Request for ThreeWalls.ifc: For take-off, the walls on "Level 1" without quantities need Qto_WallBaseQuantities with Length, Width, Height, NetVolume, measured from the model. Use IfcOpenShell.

First a look at what the model holds.

```python
import ifcopenshell
import ifcopenshell.util.element
import ifcopenshell.util.unit

model = ifcopenshell.open("ThreeWalls.ifc")
print(model.schema)
for unit_type in ("LENGTHUNIT", "AREAUNIT", "VOLUMEUNIT"):
    print(unit_type, ifcopenshell.util.unit.calculate_unit_scale(model, unit_type))
storey = next(s for s in model.by_type("IfcBuildingStorey") if s.Name == "Level 1")
walls = [e for e in ifcopenshell.util.element.get_decomposition(storey) if e.is_a("IfcWall")]
for e in sorted(walls, key=lambda e: e.id()):
    print(e.id(), e.is_a(), e.Name, list(ifcopenshell.util.element.get_psets(e, qtos_only=True)), sep=" | ")
```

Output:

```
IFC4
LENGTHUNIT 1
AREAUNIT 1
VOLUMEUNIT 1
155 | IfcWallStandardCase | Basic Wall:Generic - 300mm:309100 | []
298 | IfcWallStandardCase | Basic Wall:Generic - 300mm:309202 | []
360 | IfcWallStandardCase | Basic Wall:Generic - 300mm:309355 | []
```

```python
import ifcopenshell
import ifcopenshell.api.pset
import ifcopenshell.geom
import ifcopenshell.util.element
import ifcopenshell.util.shape
import ifcopenshell.util.unit

model = ifcopenshell.open("ThreeWalls.ifc")
unit_scale = ifcopenshell.util.unit.calculate_unit_scale(model)
volume_scale = ifcopenshell.util.unit.calculate_unit_scale(model, "VOLUMEUNIT")
settings = ifcopenshell.geom.settings()

storey = next(s for s in model.by_type("IfcBuildingStorey") if s.Name == "Level 1")
walls = [e for e in ifcopenshell.util.element.get_decomposition(storey) if e.is_a("IfcWall")]

for e in sorted(walls, key=lambda e: e.id()):
    if ifcopenshell.util.element.get_psets(e, qtos_only=True, should_inherit=False):
        continue
    # Geometry comes back in metres, in the element's own axes.
    shape = ifcopenshell.geom.create_shape(settings, e)
    values = {
        "Length": ifcopenshell.util.shape.get_x(shape.geometry) / unit_scale,
        "Width": ifcopenshell.util.shape.get_y(shape.geometry) / unit_scale,
        "Height": ifcopenshell.util.shape.get_z(shape.geometry) / unit_scale,
        "NetVolume": ifcopenshell.util.shape.get_volume(shape.geometry) / volume_scale,
    }
    qto = ifcopenshell.api.pset.add_qto(model, product=e, name="Qto_WallBaseQuantities")
    ifcopenshell.api.pset.edit_qto(model, qto=qto, properties=values)
    print(e.id(), {k: round(v, 3) for k, v in values.items()})

model.write("ThreeWalls_v2.ifc")
```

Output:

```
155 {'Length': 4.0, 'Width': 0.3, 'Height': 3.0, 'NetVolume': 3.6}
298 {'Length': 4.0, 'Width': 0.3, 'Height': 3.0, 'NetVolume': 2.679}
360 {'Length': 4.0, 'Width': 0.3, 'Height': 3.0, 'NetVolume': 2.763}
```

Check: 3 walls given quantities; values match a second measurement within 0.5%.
